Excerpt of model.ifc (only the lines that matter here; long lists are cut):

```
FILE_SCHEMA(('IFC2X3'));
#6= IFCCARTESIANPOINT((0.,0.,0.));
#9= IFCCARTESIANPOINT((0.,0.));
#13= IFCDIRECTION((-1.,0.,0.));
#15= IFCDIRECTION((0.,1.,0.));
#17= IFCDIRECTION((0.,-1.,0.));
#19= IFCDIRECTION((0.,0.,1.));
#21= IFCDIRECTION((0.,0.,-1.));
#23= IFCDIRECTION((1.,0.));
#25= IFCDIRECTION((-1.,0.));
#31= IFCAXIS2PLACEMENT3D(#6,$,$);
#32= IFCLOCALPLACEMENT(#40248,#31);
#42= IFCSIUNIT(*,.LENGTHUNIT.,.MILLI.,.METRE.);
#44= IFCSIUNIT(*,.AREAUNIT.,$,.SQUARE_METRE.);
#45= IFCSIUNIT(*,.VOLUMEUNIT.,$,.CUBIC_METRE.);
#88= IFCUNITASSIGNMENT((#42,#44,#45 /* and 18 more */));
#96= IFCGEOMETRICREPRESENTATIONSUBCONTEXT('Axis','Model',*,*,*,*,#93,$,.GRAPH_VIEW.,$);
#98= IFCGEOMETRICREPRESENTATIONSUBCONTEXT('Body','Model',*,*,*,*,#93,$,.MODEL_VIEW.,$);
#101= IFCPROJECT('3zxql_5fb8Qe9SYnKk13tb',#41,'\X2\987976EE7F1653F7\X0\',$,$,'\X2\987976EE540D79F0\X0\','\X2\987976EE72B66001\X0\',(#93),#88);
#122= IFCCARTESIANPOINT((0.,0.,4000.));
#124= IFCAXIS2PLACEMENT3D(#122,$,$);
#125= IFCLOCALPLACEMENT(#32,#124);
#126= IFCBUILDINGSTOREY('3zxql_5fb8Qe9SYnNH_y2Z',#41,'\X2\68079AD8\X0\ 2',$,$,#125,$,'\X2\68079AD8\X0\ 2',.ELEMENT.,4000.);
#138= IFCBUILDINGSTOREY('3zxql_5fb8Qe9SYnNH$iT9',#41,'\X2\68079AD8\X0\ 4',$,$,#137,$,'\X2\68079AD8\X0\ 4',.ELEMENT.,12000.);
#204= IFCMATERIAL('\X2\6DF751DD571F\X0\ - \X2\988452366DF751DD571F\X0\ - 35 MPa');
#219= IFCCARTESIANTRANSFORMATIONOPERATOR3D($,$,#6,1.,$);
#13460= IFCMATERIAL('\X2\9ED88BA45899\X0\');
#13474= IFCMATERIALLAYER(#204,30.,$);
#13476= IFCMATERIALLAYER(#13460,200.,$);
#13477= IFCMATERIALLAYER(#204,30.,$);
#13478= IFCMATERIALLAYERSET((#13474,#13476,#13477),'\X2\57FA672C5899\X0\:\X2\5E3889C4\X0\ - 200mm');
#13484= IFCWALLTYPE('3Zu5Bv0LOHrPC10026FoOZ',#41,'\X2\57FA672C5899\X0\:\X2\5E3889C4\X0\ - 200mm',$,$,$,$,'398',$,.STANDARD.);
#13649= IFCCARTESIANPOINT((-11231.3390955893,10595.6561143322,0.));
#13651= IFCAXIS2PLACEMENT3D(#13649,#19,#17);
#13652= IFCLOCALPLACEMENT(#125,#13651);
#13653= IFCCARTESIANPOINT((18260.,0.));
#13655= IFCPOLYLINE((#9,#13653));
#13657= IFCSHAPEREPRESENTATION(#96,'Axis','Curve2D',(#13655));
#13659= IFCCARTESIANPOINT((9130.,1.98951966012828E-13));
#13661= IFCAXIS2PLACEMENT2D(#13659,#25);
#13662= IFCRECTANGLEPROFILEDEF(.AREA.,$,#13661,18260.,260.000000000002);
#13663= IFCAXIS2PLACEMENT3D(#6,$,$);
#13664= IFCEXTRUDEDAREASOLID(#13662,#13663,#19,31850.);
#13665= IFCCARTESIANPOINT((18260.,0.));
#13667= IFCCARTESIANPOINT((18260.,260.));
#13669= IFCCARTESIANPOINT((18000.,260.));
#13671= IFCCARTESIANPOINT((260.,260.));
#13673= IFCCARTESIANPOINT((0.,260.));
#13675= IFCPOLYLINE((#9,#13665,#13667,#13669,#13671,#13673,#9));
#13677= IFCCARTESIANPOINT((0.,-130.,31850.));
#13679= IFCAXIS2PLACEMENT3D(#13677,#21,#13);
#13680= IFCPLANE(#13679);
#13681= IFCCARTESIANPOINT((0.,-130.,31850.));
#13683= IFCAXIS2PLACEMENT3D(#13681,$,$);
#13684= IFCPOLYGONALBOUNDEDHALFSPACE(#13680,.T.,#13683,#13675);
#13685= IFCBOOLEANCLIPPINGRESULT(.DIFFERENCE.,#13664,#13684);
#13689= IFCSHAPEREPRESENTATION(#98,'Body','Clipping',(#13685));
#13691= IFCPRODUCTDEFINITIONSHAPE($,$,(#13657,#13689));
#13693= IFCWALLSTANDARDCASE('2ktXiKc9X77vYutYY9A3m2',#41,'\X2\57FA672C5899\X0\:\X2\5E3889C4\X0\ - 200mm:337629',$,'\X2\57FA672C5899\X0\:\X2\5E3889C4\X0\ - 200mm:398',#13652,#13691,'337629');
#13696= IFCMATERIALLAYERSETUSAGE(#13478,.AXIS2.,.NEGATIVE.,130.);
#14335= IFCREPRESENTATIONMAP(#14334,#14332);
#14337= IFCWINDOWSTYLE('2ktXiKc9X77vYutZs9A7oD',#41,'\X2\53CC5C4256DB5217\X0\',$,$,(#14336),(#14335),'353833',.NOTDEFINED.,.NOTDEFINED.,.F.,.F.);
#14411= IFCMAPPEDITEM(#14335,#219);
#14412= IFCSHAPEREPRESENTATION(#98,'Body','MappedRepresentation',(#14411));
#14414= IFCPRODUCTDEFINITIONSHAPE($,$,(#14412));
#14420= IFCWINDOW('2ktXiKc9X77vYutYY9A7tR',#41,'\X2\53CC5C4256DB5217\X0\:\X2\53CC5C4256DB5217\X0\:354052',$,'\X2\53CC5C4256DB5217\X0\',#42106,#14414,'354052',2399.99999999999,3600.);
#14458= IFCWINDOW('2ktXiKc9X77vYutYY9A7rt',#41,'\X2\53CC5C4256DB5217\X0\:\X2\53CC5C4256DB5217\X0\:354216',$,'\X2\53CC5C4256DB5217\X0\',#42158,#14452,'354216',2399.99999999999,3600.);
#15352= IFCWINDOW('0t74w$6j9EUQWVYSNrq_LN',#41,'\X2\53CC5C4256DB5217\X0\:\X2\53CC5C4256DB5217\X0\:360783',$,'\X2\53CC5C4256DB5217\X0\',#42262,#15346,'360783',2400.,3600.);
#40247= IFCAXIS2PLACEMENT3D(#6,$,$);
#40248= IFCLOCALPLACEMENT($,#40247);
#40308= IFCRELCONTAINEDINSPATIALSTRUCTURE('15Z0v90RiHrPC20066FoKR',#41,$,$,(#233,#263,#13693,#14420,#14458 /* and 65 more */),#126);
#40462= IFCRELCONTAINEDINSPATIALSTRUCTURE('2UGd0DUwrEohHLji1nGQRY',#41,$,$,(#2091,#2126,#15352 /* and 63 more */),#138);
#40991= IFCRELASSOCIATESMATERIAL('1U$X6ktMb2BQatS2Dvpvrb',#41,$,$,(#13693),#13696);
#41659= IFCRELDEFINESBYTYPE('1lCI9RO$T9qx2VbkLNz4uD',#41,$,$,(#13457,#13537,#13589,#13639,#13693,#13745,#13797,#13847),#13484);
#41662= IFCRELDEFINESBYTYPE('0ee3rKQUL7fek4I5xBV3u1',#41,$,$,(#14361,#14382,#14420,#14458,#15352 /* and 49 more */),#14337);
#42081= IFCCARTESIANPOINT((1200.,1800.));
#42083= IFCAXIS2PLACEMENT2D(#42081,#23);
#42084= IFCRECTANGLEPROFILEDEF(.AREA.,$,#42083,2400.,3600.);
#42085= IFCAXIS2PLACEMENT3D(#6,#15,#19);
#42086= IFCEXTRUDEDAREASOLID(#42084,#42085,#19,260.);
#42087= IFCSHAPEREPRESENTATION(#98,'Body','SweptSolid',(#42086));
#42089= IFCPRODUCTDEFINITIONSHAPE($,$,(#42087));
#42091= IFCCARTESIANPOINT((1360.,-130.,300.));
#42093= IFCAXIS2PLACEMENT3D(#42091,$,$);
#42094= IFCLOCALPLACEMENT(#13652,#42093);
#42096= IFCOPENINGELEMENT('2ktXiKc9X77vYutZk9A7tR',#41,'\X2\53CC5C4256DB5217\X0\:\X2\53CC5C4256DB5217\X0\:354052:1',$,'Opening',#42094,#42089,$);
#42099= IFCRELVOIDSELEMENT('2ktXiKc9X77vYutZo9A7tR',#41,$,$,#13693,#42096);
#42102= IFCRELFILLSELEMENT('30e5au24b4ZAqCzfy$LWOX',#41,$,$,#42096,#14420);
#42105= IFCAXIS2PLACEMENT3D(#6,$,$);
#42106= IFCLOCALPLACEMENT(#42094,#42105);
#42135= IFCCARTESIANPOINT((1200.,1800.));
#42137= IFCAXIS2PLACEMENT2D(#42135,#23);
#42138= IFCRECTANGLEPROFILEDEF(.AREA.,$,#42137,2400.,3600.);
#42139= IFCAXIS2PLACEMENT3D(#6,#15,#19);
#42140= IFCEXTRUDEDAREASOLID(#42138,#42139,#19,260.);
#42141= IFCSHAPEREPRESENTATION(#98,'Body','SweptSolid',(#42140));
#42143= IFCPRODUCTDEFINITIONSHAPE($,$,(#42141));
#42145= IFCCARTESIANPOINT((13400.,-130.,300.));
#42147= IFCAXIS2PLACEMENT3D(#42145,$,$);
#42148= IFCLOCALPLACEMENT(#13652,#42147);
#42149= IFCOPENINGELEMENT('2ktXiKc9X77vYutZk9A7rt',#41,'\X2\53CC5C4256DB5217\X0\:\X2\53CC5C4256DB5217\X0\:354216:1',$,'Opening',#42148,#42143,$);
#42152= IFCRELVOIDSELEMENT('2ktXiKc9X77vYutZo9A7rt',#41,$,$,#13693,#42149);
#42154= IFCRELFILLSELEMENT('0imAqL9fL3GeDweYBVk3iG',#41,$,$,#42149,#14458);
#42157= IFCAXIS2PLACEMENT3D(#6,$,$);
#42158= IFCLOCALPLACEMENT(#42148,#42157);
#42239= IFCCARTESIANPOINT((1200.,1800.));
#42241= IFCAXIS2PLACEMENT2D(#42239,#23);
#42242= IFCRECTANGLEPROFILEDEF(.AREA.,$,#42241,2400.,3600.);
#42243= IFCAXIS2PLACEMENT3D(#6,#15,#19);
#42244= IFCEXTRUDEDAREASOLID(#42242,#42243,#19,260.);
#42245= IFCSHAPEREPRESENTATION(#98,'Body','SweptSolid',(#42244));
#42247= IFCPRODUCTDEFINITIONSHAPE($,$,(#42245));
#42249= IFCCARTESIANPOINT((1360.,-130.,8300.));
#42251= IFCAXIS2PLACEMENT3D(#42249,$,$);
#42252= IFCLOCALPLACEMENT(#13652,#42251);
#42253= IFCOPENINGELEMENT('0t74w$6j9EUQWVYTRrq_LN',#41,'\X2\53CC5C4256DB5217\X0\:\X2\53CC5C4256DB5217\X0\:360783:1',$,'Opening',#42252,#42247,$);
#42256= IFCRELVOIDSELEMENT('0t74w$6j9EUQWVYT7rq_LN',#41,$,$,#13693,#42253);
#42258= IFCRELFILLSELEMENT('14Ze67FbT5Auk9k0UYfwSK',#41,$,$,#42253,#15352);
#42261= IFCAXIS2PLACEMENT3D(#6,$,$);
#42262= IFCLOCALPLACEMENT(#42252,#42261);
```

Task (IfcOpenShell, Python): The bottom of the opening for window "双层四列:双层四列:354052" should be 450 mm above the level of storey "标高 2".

```python
import numpy as np
import ifcopenshell
import ifcopenshell.api.geometry
import ifcopenshell.geom
import ifcopenshell.util.element
import ifcopenshell.util.placement
import ifcopenshell.util.shape
import ifcopenshell.util.unit

model = ifcopenshell.open("model.ifc")
unit_scale = ifcopenshell.util.unit.calculate_unit_scale(model)

window = model.by_guid("2ktXiKc9X77vYutYY9A7tR")
opening = window.FillsVoids[0].RelatingOpeningElement
storey = ifcopenshell.util.element.get_container(window, ifc_class="IfcBuildingStorey")
level = ifcopenshell.util.placement.get_local_placement(storey.ObjectPlacement)[2, 3]

# The opening's origin need not be at the sill, so measure its lowest point.
shape = ifcopenshell.geom.create_shape(ifcopenshell.geom.settings(), opening)
bottom = ifcopenshell.util.shape.get_shape_bottom_elevation(shape, shape.geometry) / unit_scale
dz = level + 450.0 - bottom

shift = np.array([0.0, 0.0, dz])
# The window is placed relative to its opening, so it follows when the opening moves.
matrix = ifcopenshell.util.placement.get_local_placement(opening.ObjectPlacement)
matrix[:3, 3] += shift
ifcopenshell.api.geometry.edit_object_placement(
    model, product=opening, matrix=matrix, is_si=False, should_transform_children=True
)

print(f"moved by {dz * unit_scale:+.3f} m")

model.write("model_v2.ifc")
```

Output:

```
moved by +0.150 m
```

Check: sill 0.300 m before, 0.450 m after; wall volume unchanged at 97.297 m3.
